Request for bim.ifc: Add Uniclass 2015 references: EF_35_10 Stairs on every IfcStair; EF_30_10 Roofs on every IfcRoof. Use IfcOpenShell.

First a look at what the model holds.

```python
import ifcopenshell

model = ifcopenshell.open("bim.ifc")
print(model.schema)
print("classifications:", [c.Name for c in model.by_type("IfcClassification")])
for ifc_class in ("IfcDoor", "IfcRoof", "IfcStair", "IfcWall", "IfcWindow"):
    print(ifc_class, len(model.by_type(ifc_class)))
```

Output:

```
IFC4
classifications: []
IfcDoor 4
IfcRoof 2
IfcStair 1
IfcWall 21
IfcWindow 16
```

```python
import ifcopenshell
import ifcopenshell.api.classification

model = ifcopenshell.open("bim.ifc")

system = ifcopenshell.api.classification.add_classification(model, classification="Uniclass 2015")

codes = {
    "IfcStair": ("EF_35_10", "Stairs"),
    "IfcRoof": ("EF_30_10", "Roofs"),
}
for ifc_class, (code, name) in codes.items():
    products = model.by_type(ifc_class)
    ifcopenshell.api.classification.add_reference(
        model, products=products, classification=system, identification=code, name=name
    )
    print(code, len(products))

model.write("bim_updated.ifc")
```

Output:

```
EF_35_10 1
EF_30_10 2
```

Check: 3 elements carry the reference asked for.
